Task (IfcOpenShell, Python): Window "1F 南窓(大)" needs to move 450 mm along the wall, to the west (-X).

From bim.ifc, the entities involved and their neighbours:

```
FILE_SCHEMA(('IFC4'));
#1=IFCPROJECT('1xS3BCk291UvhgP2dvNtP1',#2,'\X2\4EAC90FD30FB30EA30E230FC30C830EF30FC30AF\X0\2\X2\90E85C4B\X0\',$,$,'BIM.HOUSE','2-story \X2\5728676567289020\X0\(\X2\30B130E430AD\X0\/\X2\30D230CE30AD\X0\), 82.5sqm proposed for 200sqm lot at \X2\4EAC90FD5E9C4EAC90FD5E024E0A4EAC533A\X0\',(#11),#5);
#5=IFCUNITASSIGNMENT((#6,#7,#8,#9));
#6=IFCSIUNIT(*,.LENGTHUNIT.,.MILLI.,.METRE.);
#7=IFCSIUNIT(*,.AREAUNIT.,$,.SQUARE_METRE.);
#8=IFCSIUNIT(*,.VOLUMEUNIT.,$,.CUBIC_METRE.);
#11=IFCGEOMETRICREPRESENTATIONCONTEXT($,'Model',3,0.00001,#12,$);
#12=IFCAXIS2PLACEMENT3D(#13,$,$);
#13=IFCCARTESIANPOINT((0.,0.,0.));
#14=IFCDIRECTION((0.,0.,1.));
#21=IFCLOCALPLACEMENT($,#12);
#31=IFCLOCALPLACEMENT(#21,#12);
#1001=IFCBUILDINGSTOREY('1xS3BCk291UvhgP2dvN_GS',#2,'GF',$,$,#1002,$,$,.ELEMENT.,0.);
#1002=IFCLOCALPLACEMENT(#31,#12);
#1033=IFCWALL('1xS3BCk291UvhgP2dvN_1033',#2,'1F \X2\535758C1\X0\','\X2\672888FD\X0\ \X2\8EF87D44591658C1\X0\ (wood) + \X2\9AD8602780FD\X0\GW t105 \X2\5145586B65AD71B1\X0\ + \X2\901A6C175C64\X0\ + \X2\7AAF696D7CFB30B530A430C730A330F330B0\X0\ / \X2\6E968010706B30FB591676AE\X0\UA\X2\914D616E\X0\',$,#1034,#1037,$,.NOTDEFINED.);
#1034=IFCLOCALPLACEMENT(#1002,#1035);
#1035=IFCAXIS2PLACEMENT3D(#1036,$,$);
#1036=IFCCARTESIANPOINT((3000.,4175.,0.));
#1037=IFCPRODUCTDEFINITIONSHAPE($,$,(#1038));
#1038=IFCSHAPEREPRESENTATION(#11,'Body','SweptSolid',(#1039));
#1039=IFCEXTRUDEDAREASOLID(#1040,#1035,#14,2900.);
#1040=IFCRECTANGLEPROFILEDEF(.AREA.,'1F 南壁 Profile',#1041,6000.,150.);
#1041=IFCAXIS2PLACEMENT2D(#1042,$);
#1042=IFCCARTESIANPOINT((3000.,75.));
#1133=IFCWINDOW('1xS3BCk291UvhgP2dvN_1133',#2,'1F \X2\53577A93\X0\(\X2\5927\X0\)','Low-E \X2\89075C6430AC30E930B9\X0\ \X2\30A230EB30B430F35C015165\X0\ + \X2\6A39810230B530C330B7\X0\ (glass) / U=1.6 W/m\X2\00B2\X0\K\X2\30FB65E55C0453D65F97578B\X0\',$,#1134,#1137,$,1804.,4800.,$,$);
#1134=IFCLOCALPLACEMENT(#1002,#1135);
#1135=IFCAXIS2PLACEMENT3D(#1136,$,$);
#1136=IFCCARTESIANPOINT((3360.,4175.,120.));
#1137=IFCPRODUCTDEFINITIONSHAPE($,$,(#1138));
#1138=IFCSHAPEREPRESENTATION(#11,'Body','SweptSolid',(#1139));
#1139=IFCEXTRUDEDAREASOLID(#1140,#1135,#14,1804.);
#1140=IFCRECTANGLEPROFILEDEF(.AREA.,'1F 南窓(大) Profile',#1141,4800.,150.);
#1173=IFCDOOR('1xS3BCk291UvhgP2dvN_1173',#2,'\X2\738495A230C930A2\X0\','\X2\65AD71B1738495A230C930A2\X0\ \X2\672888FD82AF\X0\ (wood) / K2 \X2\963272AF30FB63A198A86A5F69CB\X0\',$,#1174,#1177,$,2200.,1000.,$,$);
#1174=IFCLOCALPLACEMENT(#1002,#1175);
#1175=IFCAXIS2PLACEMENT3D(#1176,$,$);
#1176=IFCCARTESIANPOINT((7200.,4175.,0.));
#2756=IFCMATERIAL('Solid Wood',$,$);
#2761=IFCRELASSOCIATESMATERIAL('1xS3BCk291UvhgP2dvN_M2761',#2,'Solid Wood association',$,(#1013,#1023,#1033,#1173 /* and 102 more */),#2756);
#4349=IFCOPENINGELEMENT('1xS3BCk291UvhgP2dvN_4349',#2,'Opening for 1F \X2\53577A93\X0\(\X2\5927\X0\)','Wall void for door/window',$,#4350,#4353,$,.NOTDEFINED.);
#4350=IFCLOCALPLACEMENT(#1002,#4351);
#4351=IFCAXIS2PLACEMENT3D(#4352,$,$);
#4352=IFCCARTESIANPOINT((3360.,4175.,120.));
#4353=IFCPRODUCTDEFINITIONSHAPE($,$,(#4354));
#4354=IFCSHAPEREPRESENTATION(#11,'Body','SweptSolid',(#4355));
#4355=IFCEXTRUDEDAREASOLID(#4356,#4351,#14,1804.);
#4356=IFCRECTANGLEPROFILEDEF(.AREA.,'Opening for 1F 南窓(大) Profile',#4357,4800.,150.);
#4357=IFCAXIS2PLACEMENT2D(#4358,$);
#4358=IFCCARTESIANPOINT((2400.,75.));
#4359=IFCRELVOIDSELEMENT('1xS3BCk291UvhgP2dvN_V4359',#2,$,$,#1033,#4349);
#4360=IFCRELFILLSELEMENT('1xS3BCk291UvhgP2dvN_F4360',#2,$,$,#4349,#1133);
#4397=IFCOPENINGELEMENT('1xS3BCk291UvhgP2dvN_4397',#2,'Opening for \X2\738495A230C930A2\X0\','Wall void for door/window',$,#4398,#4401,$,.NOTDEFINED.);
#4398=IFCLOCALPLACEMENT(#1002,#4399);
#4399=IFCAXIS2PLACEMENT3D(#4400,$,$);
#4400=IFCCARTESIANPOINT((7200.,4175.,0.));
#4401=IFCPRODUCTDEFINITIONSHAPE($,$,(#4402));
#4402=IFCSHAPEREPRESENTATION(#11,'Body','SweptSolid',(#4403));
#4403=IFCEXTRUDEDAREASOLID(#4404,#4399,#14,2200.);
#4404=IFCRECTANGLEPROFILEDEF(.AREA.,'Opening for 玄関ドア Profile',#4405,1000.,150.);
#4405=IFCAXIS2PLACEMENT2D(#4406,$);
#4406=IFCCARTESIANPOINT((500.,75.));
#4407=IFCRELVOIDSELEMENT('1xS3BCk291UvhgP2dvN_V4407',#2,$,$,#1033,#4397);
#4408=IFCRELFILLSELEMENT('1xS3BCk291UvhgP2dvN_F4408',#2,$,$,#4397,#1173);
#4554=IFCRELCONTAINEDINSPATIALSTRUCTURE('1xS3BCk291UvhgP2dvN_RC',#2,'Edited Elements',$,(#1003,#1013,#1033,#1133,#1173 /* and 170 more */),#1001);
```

```python
import ifcopenshell
import ifcopenshell.api.geometry
import ifcopenshell.util.placement
import ifcopenshell.util.unit

model = ifcopenshell.open("bim.ifc")
unit_scale = ifcopenshell.util.unit.calculate_unit_scale(model)

window = model.by_id(1133)
opening = window.FillsVoids[0].RelatingOpeningElement
wall = opening.VoidsElements[0].RelatingBuildingElement

wall_matrix = ifcopenshell.util.placement.get_local_placement(wall.ObjectPlacement)
shift = wall_matrix[:3, 0] * -0.45 / unit_scale
before = ifcopenshell.util.placement.get_local_placement(window.ObjectPlacement)[:3, 3].copy()

# The window is not placed relative to its opening, so move both.
for product in (opening, window):
    matrix = ifcopenshell.util.placement.get_local_placement(product.ObjectPlacement)
    matrix[:3, 3] += shift
    ifcopenshell.api.geometry.edit_object_placement(model, product=product, matrix=matrix, is_si=False)

after = ifcopenshell.util.placement.get_local_placement(window.ObjectPlacement)[:3, 3]
print("window moved by", (after - before).round(3) + 0.0)

model.write("bim-out.ifc")
```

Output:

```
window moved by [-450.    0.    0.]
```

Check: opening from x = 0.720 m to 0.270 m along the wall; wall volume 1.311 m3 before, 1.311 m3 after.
